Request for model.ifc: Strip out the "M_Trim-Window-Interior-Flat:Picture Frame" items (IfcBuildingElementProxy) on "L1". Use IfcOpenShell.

First a look at what the model holds.

```python
import ifcopenshell
import ifcopenshell.util.element

model = ifcopenshell.open("model.ifc")
print(model.schema)
storey = next(s for s in model.by_type("IfcBuildingStorey") if s.Name == "L1")
proxies = [e for e in ifcopenshell.util.element.get_decomposition(storey) if e.is_a("IfcBuildingElementProxy")]
seen = {}
for e in proxies:
    element_type = ifcopenshell.util.element.get_type(e)
    name = element_type.Name if element_type not in (None, e) else None
    seen[name] = seen.get(name, 0) + 1
for name, count in sorted(seen.items(), key=str):
    print(count, "x", name)
```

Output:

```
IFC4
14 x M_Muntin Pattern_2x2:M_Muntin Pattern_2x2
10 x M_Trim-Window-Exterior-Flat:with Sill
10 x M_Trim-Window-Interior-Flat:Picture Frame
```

```python
import ifcopenshell
import ifcopenshell.api.root
import ifcopenshell.util.element

model = ifcopenshell.open("model.ifc")

storey = next(s for s in model.by_type("IfcBuildingStorey") if s.Name == "L1")
proxies = [e for e in ifcopenshell.util.element.get_decomposition(storey) if e.is_a("IfcBuildingElementProxy")]
targets = [e for e in proxies if (t := ifcopenshell.util.element.get_type(e)) not in (None, e) and t.Name == "M_Trim-Window-Interior-Flat:Picture Frame"]

for e in targets:
    ifcopenshell.api.root.remove_product(model, product=e)
print(len(targets), "removed")

model.write("model_edited.ifc")
```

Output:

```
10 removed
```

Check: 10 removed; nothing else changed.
